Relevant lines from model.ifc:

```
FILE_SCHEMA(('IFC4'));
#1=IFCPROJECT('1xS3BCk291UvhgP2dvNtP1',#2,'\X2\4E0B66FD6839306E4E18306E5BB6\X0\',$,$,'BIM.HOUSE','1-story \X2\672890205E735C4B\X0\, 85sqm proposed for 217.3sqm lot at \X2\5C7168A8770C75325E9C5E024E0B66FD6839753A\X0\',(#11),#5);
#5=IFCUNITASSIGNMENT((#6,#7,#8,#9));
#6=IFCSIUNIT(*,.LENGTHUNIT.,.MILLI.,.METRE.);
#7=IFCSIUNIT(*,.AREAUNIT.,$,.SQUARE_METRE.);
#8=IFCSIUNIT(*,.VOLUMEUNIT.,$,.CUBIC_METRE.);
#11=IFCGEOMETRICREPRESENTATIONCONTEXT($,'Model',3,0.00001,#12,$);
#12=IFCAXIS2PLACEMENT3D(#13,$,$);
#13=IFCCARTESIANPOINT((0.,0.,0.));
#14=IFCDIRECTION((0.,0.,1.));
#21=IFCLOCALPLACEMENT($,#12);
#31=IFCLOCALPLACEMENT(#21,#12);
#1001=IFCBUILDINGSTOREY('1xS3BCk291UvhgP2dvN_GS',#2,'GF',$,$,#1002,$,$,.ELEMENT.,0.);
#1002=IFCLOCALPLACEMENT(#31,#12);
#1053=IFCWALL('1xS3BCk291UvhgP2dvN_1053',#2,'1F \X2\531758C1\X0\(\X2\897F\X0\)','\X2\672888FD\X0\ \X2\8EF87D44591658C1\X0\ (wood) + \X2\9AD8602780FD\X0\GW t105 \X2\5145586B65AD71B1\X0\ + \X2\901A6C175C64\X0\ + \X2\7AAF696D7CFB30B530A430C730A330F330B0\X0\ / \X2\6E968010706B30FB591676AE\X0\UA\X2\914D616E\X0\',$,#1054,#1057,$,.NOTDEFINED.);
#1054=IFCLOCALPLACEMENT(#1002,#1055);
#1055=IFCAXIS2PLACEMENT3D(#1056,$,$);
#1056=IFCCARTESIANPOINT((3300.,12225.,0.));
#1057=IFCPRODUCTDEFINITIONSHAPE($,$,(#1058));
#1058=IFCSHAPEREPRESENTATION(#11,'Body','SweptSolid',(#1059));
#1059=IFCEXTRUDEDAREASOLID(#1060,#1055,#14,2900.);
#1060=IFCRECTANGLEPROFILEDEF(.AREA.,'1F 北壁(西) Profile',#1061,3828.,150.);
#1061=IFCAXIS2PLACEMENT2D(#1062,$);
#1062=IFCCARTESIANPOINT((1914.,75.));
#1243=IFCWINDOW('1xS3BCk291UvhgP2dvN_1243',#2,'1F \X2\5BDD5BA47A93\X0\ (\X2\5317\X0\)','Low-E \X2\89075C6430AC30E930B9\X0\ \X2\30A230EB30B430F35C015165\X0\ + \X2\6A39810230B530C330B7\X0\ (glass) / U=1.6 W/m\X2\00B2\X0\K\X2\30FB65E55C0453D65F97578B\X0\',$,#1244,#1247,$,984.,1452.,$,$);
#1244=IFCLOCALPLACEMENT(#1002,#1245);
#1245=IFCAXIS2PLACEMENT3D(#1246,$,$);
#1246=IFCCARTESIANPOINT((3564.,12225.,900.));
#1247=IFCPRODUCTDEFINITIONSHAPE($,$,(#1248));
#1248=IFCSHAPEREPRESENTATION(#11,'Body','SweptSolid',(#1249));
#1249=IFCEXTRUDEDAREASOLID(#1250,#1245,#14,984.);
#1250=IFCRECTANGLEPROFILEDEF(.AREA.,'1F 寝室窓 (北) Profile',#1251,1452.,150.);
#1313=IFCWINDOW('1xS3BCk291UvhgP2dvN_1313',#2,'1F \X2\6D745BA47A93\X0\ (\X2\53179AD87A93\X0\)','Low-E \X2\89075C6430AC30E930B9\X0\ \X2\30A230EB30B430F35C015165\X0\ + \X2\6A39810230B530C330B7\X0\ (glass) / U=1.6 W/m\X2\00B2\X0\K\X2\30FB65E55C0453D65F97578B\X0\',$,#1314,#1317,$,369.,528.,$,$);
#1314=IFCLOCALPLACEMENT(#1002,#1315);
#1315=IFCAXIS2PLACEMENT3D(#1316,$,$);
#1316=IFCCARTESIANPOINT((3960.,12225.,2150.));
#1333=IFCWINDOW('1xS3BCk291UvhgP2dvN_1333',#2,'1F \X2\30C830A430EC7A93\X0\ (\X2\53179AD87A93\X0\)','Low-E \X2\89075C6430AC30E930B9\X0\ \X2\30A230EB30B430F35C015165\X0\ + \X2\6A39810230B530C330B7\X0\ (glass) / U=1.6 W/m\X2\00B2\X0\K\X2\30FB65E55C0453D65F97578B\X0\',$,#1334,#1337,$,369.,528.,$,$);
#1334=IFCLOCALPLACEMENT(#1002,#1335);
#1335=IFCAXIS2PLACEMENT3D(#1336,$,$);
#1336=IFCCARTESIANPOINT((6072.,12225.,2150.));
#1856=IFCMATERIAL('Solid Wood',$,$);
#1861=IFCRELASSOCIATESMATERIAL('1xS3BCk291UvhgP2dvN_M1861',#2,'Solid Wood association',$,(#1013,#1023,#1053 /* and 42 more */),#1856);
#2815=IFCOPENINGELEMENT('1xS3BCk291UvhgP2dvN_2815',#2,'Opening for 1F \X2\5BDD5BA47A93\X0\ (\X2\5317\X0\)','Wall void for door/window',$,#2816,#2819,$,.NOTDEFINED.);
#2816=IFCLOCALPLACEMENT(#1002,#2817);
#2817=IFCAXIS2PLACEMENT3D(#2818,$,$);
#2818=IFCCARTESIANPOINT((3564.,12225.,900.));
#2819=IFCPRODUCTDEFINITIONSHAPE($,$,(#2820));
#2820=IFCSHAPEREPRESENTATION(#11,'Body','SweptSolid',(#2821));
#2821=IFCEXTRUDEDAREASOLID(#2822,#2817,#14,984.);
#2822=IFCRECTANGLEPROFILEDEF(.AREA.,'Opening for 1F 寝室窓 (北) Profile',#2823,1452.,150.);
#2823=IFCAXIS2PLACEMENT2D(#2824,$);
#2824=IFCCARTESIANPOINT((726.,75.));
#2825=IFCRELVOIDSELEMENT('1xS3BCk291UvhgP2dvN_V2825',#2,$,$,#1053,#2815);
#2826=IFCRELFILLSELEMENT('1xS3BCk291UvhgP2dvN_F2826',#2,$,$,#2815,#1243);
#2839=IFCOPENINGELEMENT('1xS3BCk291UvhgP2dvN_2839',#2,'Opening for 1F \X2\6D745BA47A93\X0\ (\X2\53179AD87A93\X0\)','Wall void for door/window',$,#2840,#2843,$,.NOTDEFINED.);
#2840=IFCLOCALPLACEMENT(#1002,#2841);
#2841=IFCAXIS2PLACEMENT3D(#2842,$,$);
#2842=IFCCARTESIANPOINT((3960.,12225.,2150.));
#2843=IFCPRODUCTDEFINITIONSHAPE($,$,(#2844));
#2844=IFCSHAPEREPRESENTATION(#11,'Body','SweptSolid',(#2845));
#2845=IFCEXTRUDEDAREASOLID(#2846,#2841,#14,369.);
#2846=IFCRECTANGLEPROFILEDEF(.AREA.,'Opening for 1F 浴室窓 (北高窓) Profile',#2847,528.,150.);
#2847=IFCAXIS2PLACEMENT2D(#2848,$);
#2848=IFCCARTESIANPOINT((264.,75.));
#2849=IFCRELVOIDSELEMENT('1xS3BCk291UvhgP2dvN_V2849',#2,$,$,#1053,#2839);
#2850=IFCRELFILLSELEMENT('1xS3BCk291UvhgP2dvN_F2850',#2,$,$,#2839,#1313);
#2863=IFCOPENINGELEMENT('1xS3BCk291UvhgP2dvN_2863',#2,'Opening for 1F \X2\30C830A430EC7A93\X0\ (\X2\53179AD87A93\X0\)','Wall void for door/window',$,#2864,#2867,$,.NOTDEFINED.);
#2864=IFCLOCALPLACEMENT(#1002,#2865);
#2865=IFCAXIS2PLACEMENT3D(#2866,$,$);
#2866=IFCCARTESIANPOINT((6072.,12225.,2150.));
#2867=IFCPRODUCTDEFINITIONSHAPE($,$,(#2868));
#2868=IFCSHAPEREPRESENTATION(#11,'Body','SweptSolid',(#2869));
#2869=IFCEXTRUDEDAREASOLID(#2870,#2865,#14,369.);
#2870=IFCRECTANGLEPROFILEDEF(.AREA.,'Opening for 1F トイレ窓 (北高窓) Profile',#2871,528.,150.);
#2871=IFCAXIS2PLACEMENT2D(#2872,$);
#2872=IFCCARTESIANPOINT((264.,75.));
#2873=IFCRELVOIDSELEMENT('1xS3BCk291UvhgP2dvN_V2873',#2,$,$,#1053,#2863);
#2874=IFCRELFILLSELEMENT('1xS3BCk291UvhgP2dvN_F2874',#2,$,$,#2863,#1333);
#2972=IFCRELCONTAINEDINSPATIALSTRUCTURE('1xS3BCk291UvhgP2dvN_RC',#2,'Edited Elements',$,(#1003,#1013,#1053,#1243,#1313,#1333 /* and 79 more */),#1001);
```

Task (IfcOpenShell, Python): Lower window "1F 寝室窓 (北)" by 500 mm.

```python
import numpy as np
import ifcopenshell
import ifcopenshell.api.geometry
import ifcopenshell.util.placement
import ifcopenshell.util.unit

model = ifcopenshell.open("model.ifc")
unit_scale = ifcopenshell.util.unit.calculate_unit_scale(model)

window = model.by_guid("1xS3BCk291UvhgP2dvN_1243")
opening = window.FillsVoids[0].RelatingOpeningElement
dz = -500.0

shift = np.array([0.0, 0.0, dz])
# The window is not placed relative to its opening, so move both.
for product in (opening, window):
    matrix = ifcopenshell.util.placement.get_local_placement(product.ObjectPlacement)
    matrix[:3, 3] += shift
    ifcopenshell.api.geometry.edit_object_placement(model, product=product, matrix=matrix, is_si=False)

print(f"moved by {dz * unit_scale:+.3f} m")

model.write("model_v2.ifc")
```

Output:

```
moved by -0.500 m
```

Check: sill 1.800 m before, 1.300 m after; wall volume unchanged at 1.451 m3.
